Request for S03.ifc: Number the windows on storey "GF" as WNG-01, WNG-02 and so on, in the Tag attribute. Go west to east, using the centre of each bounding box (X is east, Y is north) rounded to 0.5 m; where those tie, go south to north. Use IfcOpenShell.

First a look at what the model holds.

```python
import ifcopenshell
import ifcopenshell.util.element
import ifcopenshell.util.placement

model = ifcopenshell.open("S03.ifc")
print(model.schema)
storey = next(s for s in model.by_type("IfcBuildingStorey") if s.Name == "GF")
windows = [e for e in ifcopenshell.util.element.get_decomposition(storey) if e.is_a("IfcWindow")]
for e in sorted(windows, key=lambda e: e.id()):
    origin = ifcopenshell.util.placement.get_local_placement(e.ObjectPlacement)[:3, 3]
    print(e.id(), e.Tag, e.Name, origin.round(2) + 0.0, sep=" | ")
```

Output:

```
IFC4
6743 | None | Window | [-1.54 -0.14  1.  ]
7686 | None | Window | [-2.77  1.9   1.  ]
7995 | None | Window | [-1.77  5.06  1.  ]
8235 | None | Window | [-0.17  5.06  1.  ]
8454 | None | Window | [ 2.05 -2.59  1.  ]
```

```python
import ifcopenshell
import ifcopenshell.geom
import ifcopenshell.util.element
import ifcopenshell.util.shape

model = ifcopenshell.open("S03.ifc")
settings = ifcopenshell.geom.settings()
settings.set("use-world-coords", True)


def centre(element):
    shape = ifcopenshell.geom.create_shape(settings, element)
    return ifcopenshell.util.shape.get_bbox_centroid(shape.geometry)


storey = next(s for s in model.by_type("IfcBuildingStorey") if s.Name == "GF")
windows = [e for e in ifcopenshell.util.element.get_decomposition(storey) if e.is_a("IfcWindow")]

# Insertion points can sit at a corner or the storey origin, so sort by the geometry (in metres).
centres = {e: centre(e) for e in windows}
windows.sort(key=lambda e: (round(centres[e][0] / 0.5), centres[e][1]))

for i, e in enumerate(windows, start=1):
    number = f"WNG-{i:02d}"
    e.Tag = number
    print(e.id(), number)

model.write("S03_v2.ifc")
```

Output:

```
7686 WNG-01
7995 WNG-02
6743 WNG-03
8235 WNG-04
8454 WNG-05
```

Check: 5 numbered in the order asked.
